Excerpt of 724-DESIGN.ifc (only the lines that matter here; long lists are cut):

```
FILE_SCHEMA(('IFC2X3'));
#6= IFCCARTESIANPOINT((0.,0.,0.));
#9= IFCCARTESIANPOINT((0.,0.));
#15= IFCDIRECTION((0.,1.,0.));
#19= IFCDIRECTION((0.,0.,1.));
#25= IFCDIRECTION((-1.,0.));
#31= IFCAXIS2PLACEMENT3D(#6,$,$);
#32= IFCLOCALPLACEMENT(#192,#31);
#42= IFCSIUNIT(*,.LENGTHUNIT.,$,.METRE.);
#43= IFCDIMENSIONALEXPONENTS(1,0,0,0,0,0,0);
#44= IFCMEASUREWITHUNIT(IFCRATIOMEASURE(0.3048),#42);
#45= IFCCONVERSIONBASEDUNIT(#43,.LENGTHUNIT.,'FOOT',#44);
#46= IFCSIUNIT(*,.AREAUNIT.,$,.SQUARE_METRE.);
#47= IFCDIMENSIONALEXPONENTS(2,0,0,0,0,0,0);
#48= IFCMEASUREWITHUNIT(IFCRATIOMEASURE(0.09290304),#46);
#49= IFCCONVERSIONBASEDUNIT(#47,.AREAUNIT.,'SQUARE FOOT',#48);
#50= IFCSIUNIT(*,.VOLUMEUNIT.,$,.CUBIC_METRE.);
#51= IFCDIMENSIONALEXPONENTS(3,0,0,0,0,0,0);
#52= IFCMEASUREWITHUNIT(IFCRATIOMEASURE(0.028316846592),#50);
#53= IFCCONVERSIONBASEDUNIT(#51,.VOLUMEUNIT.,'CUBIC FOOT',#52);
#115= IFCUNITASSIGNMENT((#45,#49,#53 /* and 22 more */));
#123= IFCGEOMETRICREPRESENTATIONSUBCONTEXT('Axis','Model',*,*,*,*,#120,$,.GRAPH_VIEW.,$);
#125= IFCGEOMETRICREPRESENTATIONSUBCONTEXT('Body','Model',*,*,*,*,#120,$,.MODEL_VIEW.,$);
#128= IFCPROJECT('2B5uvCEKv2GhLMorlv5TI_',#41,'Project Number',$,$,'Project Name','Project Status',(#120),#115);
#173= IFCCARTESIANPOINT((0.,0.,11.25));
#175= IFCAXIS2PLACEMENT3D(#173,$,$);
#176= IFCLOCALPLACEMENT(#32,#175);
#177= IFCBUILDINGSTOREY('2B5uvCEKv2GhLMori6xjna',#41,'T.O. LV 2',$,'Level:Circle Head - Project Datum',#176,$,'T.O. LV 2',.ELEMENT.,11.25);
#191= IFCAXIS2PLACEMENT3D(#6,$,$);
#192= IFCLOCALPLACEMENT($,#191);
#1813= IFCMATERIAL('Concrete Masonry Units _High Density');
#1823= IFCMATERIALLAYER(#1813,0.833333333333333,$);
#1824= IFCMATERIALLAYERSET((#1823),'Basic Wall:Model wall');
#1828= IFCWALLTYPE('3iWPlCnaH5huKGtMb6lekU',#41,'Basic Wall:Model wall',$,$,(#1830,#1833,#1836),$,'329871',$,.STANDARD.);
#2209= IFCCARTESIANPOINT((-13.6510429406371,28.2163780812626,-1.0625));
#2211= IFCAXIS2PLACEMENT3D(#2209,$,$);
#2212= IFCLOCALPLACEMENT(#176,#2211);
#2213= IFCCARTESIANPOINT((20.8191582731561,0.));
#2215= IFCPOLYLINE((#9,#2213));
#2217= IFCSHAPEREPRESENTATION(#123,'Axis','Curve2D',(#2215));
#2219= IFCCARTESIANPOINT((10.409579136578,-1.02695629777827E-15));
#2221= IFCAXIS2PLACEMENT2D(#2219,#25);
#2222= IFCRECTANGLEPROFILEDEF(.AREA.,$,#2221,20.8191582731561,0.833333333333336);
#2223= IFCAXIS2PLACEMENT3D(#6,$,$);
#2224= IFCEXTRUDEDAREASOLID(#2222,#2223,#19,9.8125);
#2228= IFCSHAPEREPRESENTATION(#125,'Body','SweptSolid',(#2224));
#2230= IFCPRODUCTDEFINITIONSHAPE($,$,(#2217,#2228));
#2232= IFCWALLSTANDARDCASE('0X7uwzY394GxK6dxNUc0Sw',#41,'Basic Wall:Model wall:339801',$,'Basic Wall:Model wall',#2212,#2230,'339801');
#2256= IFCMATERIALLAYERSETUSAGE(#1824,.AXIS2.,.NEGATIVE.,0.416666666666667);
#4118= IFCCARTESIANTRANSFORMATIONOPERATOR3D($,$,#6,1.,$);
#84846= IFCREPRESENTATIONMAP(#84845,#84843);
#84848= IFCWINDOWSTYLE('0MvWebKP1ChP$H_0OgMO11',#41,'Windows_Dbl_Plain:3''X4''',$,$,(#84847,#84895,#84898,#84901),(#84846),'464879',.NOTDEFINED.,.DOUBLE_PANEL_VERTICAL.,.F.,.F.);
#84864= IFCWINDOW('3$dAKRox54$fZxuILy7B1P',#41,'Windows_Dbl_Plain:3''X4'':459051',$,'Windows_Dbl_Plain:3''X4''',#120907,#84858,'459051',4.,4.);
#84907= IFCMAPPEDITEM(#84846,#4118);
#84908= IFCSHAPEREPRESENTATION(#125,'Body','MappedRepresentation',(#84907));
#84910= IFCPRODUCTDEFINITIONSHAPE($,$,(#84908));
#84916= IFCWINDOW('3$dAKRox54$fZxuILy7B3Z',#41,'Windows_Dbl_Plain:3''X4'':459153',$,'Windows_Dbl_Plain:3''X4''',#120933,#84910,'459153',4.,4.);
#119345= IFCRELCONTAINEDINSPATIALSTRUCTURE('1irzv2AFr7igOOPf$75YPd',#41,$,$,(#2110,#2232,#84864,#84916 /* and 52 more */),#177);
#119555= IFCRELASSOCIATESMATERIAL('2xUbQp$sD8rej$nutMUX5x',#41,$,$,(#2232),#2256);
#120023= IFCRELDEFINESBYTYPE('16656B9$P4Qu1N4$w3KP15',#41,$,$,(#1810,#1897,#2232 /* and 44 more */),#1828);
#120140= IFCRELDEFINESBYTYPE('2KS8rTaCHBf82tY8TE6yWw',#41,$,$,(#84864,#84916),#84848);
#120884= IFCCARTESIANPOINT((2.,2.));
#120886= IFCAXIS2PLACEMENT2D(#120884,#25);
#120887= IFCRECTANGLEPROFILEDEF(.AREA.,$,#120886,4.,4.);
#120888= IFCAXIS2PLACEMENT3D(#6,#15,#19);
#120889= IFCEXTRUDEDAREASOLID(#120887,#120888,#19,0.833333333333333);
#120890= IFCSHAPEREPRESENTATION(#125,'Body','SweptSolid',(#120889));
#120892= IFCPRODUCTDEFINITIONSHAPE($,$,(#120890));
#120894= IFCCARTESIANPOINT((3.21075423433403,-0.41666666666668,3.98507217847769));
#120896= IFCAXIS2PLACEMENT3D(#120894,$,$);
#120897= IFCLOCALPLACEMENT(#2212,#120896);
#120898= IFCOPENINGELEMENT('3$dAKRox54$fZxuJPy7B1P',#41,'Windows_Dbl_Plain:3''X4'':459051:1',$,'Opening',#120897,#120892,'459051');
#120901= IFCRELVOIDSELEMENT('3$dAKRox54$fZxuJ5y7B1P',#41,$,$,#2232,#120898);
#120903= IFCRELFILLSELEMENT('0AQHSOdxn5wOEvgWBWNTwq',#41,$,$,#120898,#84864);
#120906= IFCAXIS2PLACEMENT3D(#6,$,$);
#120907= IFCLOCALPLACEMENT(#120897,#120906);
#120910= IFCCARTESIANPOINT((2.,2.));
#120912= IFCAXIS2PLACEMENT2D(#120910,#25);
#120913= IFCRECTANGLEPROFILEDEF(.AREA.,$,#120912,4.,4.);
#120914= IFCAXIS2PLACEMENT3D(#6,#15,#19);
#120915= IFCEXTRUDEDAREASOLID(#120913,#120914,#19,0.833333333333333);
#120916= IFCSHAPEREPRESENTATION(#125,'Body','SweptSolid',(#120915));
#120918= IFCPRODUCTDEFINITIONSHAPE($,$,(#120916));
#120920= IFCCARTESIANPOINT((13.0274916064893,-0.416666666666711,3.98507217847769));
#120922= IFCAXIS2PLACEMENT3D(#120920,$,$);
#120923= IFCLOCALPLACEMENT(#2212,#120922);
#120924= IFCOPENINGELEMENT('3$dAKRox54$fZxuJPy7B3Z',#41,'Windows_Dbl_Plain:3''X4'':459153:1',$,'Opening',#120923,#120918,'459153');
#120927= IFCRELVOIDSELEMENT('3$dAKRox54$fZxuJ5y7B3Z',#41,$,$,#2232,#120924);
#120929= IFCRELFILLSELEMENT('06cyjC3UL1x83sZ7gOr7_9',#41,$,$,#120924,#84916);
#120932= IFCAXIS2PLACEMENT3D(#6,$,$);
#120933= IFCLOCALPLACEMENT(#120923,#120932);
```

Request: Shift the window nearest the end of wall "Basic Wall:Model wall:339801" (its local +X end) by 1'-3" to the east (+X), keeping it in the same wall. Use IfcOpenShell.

```python
import ifcopenshell
import ifcopenshell.api.geometry
import ifcopenshell.util.placement
import ifcopenshell.util.unit

model = ifcopenshell.open("724-DESIGN.ifc")
unit_scale = ifcopenshell.util.unit.calculate_unit_scale(model)

window = model.by_guid("3$dAKRox54$fZxuILy7B3Z")
opening = window.FillsVoids[0].RelatingOpeningElement
wall = opening.VoidsElements[0].RelatingBuildingElement

wall_matrix = ifcopenshell.util.placement.get_local_placement(wall.ObjectPlacement)
shift = wall_matrix[:3, 0] * 15 * 0.0254 / unit_scale
before = ifcopenshell.util.placement.get_local_placement(window.ObjectPlacement)[:3, 3].copy()

# The window is placed relative to its opening, so it follows when the opening moves.
matrix = ifcopenshell.util.placement.get_local_placement(opening.ObjectPlacement)
matrix[:3, 3] += shift
ifcopenshell.api.geometry.edit_object_placement(
    model, product=opening, matrix=matrix, is_si=False, should_transform_children=True
)

after = ifcopenshell.util.placement.get_local_placement(window.ObjectPlacement)[:3, 3]
print("window moved by", (after - before).round(3) + 0.0)

model.write("724-DESIGN_rev.ifc")
```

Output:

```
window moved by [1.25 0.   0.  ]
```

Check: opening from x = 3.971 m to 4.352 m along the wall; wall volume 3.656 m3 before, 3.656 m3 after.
